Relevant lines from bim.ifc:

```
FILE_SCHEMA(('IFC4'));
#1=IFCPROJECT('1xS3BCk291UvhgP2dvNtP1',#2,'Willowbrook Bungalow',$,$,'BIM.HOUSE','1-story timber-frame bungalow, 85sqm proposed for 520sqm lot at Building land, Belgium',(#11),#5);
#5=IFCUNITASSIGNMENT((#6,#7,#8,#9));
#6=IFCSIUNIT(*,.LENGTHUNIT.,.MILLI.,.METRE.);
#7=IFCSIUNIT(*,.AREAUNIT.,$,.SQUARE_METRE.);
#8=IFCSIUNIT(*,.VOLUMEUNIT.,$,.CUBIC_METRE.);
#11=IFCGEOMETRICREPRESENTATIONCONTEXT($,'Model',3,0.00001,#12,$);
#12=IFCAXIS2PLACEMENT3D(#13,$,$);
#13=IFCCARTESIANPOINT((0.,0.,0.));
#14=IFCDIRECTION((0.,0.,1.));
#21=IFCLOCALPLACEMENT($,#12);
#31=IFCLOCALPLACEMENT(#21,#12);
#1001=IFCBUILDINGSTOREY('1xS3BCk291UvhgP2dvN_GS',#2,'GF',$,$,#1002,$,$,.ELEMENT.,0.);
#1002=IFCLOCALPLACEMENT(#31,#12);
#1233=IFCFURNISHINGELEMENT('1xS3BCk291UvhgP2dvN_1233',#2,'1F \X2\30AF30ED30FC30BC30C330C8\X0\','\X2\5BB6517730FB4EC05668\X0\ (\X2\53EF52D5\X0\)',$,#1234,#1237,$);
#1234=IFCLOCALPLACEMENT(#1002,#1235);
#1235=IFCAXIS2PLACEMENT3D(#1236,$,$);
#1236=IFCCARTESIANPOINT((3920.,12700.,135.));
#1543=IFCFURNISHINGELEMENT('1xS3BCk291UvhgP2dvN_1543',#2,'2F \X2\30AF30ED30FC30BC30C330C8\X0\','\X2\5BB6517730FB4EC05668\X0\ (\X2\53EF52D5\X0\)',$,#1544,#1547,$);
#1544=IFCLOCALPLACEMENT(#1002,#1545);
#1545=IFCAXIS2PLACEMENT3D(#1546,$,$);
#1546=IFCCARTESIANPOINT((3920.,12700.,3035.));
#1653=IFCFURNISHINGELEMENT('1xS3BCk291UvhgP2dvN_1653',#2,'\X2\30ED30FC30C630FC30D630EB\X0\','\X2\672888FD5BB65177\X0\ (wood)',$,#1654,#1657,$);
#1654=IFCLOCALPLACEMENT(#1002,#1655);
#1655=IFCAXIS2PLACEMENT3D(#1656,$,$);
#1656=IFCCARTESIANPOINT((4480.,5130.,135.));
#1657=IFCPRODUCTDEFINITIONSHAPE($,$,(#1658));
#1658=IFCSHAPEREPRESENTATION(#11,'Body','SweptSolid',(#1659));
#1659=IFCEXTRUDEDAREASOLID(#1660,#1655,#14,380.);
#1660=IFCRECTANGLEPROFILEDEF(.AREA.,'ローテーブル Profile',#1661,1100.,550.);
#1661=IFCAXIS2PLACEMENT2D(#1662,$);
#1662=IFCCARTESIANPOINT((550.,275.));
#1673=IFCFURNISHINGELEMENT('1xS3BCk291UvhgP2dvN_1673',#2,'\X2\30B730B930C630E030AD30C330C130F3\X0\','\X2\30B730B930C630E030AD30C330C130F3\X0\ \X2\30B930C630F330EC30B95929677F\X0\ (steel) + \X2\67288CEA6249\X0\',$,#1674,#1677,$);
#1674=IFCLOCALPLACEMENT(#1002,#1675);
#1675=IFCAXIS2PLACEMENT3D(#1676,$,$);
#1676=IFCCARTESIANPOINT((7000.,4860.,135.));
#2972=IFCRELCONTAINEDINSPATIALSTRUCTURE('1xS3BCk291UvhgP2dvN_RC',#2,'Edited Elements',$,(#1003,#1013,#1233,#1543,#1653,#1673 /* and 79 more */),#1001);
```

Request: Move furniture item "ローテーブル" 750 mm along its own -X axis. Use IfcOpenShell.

```python
import ifcopenshell
import ifcopenshell.api.geometry
import ifcopenshell.util.placement
import ifcopenshell.util.unit

model = ifcopenshell.open("bim.ifc")
unit_scale = ifcopenshell.util.unit.calculate_unit_scale(model)

item = model.by_id(1653)
matrix = ifcopenshell.util.placement.get_local_placement(item.ObjectPlacement)
matrix[:3, 3] -= matrix[:3, 0] * 0.75 / unit_scale
ifcopenshell.api.geometry.edit_object_placement(model, product=item, matrix=matrix, is_si=False)

print(ifcopenshell.util.placement.get_local_placement(item.ObjectPlacement).round(3) + 0.0)

model.write("bim_edited.ifc")
```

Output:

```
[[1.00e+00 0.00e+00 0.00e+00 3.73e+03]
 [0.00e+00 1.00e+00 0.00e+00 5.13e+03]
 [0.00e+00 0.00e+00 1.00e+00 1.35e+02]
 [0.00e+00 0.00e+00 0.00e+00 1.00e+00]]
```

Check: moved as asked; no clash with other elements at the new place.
